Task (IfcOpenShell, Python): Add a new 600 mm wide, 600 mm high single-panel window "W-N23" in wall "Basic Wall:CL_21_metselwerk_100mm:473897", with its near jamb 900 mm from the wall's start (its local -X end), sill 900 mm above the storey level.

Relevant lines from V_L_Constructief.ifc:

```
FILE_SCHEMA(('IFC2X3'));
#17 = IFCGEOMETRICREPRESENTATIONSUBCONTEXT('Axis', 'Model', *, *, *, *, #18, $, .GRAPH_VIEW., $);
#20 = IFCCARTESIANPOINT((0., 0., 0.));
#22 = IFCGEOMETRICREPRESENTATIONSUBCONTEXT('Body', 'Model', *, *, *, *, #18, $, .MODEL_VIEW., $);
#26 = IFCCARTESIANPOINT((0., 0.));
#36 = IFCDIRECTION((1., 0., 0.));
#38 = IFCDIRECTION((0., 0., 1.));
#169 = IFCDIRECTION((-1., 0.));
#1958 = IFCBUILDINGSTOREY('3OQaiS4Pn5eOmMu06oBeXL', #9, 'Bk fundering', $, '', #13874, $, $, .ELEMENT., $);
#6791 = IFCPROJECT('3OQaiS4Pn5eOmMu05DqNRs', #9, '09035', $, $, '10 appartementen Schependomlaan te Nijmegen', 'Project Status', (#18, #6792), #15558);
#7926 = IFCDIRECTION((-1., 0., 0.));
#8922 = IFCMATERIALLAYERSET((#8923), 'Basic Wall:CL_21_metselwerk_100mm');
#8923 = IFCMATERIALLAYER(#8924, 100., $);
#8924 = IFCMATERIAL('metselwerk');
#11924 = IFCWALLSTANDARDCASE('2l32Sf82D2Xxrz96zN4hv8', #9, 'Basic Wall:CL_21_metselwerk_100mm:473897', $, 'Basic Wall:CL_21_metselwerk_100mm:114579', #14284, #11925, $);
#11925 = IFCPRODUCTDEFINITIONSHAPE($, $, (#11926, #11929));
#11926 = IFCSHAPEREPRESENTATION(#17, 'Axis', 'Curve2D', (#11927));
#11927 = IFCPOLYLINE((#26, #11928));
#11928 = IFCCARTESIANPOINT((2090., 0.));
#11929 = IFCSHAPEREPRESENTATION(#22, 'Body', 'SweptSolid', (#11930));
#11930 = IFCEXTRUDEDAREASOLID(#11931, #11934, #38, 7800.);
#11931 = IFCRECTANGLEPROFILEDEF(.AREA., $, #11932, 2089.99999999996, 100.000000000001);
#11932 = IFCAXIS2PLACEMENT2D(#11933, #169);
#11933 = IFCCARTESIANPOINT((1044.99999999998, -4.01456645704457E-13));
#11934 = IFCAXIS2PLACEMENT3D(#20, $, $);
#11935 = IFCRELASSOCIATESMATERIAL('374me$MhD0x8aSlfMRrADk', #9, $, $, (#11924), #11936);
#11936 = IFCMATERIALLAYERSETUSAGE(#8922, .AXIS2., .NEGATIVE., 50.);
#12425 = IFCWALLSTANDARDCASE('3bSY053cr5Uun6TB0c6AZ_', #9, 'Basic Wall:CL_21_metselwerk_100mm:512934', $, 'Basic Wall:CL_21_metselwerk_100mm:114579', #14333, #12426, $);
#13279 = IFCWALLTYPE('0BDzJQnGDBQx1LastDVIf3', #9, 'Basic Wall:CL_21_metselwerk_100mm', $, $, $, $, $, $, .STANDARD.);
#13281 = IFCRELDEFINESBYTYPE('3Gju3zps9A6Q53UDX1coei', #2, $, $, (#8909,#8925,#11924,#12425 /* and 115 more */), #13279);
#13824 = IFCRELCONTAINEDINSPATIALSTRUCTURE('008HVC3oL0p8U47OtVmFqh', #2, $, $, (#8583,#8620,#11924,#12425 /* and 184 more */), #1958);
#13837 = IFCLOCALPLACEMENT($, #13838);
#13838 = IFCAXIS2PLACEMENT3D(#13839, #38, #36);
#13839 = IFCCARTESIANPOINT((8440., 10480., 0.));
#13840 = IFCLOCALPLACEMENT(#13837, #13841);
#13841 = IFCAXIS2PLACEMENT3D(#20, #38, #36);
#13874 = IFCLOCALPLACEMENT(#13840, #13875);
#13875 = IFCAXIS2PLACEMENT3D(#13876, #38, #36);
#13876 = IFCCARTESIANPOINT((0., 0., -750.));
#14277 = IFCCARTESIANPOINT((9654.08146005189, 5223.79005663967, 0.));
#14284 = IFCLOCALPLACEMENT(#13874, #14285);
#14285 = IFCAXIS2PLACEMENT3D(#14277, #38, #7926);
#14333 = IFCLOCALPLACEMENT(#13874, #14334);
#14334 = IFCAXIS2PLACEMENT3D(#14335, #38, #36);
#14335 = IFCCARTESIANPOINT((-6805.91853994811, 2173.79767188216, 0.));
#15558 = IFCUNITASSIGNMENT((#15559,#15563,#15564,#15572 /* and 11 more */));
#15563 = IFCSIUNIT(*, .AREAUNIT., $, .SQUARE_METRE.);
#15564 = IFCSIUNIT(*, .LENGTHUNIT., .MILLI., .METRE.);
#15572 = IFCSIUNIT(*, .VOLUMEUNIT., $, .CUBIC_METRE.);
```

```python
import numpy as np
import ifcopenshell
import ifcopenshell.api.feature
import ifcopenshell.api.geometry
import ifcopenshell.api.root
import ifcopenshell.api.spatial
import ifcopenshell.api.type
import ifcopenshell.geom
import ifcopenshell.util.element
import ifcopenshell.util.placement
import ifcopenshell.util.representation
import ifcopenshell.util.shape
import ifcopenshell.util.unit

model = ifcopenshell.open("V_L_Constructief.ifc")
unit_scale = ifcopenshell.util.unit.calculate_unit_scale(model)
settings = ifcopenshell.geom.settings()


def volume(element):
    """Net volume in cubic metres, openings subtracted."""
    shape = ifcopenshell.geom.create_shape(settings, element)
    return ifcopenshell.util.shape.get_volume(shape.geometry)


wall = model.by_guid("2l32Sf82D2Xxrz96zN4hv8")
storey = ifcopenshell.util.element.get_container(wall, ifc_class="IfcBuildingStorey")
context = ifcopenshell.util.representation.get_context(model, "Model", "Body", "MODEL_VIEW")
before = volume(wall)

width, height, from_end, sill = 0.6, 0.6, 0.9, 0.9  # metres

# The wall runs along its own X axis, and the end named is its -X end.
wall_shape = ifcopenshell.geom.create_shape(settings, wall)
x, y, z = ifcopenshell.util.shape.get_vertices(wall_shape.geometry).T
start = x.min() + from_end
face, thickness = float(y.min()), float(y.max() - y.min())
wall_matrix = ifcopenshell.util.placement.get_local_placement(wall.ObjectPlacement)
level = ifcopenshell.util.placement.get_local_placement(storey.ObjectPlacement)[2, 3]


def in_wall(x, y):
    """Placement at x, y metres in the wall's axes, at sill height."""
    matrix = wall_matrix.copy()
    matrix[:, 3] = wall_matrix @ np.array([x / unit_scale, y / unit_scale, 0.0, 1.0])
    matrix[2, 3] = level + sill / unit_scale
    return matrix


# Opening: a box that overshoots both wall faces by 50 mm.
opening = ifcopenshell.api.root.create_entity(model, ifc_class="IfcOpeningElement")
box = ifcopenshell.api.geometry.add_wall_representation(
    model, context=context, length=width, height=height, thickness=thickness + 0.1
)
ifcopenshell.api.geometry.assign_representation(model, product=opening, representation=box)
ifcopenshell.api.geometry.edit_object_placement(model, product=opening, matrix=in_wall(start, face - 0.05), is_si=False)
ifcopenshell.api.feature.add_feature(model, feature=opening, element=wall)

window = ifcopenshell.api.root.create_entity(model, ifc_class="IfcWindow", name="W-N23")
window.OverallWidth, window.OverallHeight = width / unit_scale, height / unit_scale
body = ifcopenshell.api.geometry.add_window_representation(
    model,
    context=context,
    overall_width=window.OverallWidth,
    overall_height=window.OverallHeight,
    partition_type="SINGLE_PANEL",
)
ifcopenshell.api.geometry.assign_representation(model, product=window, representation=body)
ifcopenshell.api.spatial.assign_container(model, products=[window], relating_structure=storey)
fills = ifcopenshell.api.feature.add_filling(model, opening=opening, element=window)
fills.OwnerHistory = window.OwnerHistory  # required in IFC2X3

# IFC2X3 keeps the operation on the window style.
style = ifcopenshell.api.root.create_entity(model, ifc_class="IfcWindowStyle", name="W-N23")
style.OperationType, style.ConstructionType = "SINGLE_PANEL", "NOTDEFINED"
style.ParameterTakesPrecedence = style.Sizeable = False
ifcopenshell.api.type.assign_type(model, related_objects=[window], relating_type=style)

# Centre the window in the wall's thickness.
ifcopenshell.api.geometry.edit_object_placement(model, product=window, matrix=in_wall(start, face), is_si=False)
window_shape = ifcopenshell.geom.create_shape(settings, window)
depth = ifcopenshell.util.shape.get_vertices(window_shape.geometry)[:, 1]
offset = face + thickness / 2 - (depth.min() + depth.max()) / 2
ifcopenshell.api.geometry.edit_object_placement(model, product=window, matrix=in_wall(start, offset), is_si=False)

after = volume(wall)

print(f"wall volume {before:.3f} -> {after:.3f} m3")

model.write("V_L_Constructief_rev.ifc")
```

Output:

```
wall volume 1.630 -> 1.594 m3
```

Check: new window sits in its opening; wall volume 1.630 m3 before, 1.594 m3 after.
